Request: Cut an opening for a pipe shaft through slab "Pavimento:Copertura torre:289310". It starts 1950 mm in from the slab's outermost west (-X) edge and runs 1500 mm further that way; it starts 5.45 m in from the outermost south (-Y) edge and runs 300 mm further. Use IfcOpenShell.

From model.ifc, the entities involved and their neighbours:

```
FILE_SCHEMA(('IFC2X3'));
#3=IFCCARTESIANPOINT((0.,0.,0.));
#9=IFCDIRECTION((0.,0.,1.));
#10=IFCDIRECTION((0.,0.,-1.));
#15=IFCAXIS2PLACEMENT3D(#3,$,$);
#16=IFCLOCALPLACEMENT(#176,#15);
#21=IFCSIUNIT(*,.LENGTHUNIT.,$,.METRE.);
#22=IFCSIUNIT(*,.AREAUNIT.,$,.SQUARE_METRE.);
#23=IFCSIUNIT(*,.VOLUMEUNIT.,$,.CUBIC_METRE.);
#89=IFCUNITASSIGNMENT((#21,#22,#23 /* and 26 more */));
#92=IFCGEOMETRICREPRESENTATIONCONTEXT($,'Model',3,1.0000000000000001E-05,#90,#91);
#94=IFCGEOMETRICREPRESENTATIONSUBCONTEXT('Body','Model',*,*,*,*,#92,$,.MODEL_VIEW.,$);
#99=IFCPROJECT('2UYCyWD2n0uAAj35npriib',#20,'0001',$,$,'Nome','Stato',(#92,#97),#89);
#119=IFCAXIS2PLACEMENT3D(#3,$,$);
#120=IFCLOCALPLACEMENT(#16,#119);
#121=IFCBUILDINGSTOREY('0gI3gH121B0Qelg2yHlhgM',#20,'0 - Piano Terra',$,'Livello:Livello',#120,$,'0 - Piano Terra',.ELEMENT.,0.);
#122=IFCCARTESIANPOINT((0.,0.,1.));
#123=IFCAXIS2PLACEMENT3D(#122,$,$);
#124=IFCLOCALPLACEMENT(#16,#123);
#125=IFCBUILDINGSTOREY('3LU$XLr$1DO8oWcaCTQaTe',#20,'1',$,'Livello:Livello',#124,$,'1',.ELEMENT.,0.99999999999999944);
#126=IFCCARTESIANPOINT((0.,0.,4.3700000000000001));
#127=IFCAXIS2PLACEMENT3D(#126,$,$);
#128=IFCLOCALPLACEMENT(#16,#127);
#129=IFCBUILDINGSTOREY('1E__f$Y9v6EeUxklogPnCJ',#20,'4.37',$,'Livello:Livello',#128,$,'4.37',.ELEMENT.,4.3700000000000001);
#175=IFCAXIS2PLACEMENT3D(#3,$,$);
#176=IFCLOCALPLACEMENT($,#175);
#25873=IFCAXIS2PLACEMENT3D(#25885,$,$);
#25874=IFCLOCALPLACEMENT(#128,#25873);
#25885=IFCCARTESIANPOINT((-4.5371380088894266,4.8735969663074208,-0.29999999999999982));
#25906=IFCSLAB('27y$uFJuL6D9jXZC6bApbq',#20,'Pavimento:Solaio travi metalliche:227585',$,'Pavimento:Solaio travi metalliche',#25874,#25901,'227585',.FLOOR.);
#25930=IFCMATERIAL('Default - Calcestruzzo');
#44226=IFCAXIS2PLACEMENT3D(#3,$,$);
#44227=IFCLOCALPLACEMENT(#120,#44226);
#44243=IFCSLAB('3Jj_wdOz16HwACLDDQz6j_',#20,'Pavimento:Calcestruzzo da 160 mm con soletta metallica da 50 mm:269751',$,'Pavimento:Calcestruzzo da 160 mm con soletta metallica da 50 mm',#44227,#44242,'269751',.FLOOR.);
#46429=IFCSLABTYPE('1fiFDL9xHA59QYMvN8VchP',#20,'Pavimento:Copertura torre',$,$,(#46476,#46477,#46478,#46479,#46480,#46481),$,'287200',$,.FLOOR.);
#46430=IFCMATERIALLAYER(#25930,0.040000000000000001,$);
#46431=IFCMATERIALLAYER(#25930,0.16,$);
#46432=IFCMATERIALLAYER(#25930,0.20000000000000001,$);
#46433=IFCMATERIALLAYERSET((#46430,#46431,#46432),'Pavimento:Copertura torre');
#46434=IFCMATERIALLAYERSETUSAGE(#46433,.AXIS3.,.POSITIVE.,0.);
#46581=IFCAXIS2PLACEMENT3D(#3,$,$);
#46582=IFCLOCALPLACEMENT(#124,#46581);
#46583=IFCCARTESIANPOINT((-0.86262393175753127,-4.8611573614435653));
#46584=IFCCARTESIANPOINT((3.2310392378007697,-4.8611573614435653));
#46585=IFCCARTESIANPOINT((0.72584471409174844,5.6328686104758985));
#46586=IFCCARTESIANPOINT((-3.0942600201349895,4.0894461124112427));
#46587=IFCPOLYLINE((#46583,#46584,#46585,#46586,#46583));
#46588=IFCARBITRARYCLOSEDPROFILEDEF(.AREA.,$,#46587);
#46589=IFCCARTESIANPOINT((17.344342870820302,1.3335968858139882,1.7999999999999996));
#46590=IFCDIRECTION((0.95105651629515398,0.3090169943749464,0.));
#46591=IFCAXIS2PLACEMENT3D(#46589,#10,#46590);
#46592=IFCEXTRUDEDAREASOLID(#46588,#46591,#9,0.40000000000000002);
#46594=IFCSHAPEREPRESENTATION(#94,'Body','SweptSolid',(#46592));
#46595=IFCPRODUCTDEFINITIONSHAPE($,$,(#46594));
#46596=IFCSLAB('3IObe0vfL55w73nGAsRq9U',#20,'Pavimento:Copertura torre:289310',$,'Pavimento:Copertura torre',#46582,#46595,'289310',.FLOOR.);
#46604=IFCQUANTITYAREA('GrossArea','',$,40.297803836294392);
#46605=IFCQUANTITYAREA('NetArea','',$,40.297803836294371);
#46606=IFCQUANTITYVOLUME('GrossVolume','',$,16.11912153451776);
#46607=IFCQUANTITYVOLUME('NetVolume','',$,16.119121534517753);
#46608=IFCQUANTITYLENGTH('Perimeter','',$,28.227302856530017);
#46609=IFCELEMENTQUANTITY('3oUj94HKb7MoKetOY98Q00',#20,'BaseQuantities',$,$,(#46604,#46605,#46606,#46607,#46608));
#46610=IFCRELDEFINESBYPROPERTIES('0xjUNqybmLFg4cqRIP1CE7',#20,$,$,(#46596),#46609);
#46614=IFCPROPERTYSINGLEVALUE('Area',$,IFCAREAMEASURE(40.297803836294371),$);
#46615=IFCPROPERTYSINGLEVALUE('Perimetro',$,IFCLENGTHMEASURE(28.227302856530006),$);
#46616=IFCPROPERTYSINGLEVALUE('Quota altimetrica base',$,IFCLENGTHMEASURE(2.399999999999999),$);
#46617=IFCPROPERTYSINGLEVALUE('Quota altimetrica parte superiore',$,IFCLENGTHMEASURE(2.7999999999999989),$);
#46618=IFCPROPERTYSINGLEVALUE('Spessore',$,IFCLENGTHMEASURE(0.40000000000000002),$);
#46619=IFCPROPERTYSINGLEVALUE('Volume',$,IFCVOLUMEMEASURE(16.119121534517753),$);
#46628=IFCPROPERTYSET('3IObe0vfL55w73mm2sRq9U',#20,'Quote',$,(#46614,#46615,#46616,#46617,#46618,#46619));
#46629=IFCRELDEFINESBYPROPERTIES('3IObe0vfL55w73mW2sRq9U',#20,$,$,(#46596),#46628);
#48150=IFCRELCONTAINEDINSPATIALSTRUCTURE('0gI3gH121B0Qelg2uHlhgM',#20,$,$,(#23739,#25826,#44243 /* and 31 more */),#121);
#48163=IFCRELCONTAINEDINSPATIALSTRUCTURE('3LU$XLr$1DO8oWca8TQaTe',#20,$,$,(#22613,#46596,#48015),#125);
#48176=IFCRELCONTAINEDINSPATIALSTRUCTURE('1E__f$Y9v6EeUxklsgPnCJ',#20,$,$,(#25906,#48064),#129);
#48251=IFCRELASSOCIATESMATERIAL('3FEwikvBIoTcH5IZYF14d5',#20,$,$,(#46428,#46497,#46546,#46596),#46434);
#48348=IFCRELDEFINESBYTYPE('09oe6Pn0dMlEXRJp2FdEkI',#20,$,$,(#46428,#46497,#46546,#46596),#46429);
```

```python
import numpy as np
import ifcopenshell
import ifcopenshell.api.feature
import ifcopenshell.api.geometry
import ifcopenshell.api.pset
import ifcopenshell.api.root
import ifcopenshell.geom
import ifcopenshell.util.element
import ifcopenshell.util.placement
import ifcopenshell.util.representation
import ifcopenshell.util.shape
import ifcopenshell.util.unit

model = ifcopenshell.open("model.ifc")
unit_scale = ifcopenshell.util.unit.calculate_unit_scale(model)
area_scale = ifcopenshell.util.unit.calculate_unit_scale(model, "AREAUNIT")
volume_scale = ifcopenshell.util.unit.calculate_unit_scale(model, "VOLUMEUNIT")
settings = ifcopenshell.geom.settings()


def volume(element):
    """Net volume in cubic metres, openings subtracted."""
    shape = ifcopenshell.geom.create_shape(settings, element)
    return ifcopenshell.util.shape.get_volume(shape.geometry)


slab = model.by_guid("3IObe0vfL55w73nGAsRq9U")
before = volume(slab)

# Extent in the slab's own axes, in metres. The edges named are its -X and -Y sides.
slab_shape = ifcopenshell.geom.create_shape(settings, slab)
vertices = ifcopenshell.util.shape.get_vertices(slab_shape.geometry)
x_min, y_min, bottom = vertices.min(axis=0)
top = vertices[:, 2].max()

opening = ifcopenshell.api.root.create_entity(model, ifc_class="IfcOpeningElement", name="Pipe shaft opening")
context = ifcopenshell.util.representation.get_context(model, "Model", "Body", "MODEL_VIEW")
width, depth = 1.5, 0.3
outline = [(0.0, 0.0), (width, 0.0), (width, depth), (0.0, depth), (0.0, 0.0)]
# Overshoot both faces by 50 mm so the cut is clean.
shape = ifcopenshell.api.geometry.add_slab_representation(
    model, context=context, depth=top - bottom + 0.1, polyline=outline
)
ifcopenshell.api.geometry.assign_representation(model, product=opening, representation=shape)

matrix = ifcopenshell.util.placement.get_local_placement(slab.ObjectPlacement)
matrix[:, 3] = matrix @ np.append(np.array([x_min + 1.95, y_min + 5.45, bottom - 0.05]) / unit_scale, 1.0)
ifcopenshell.api.geometry.edit_object_placement(model, product=opening, matrix=matrix, is_si=False)
ifcopenshell.api.feature.add_feature(model, feature=opening, element=slab)

after = volume(slab)

# Update the slab's stored quantities.
qto = model.by_id(ifcopenshell.util.element.get_pset(slab, "BaseQuantities", should_inherit=False)["id"])
ifcopenshell.api.pset.edit_qto(model, qto=qto, properties={
    "NetArea": after / (top - bottom) / area_scale,
    "NetVolume": after / volume_scale,
})
pset = model.by_id(ifcopenshell.util.element.get_pset(slab, "Quote", should_inherit=False)["id"])
ifcopenshell.api.pset.edit_pset(model, pset=pset, properties={
    "Area": model.create_entity("IfcAreaMeasure", after / (top - bottom) / area_scale),
    "Volume": model.create_entity("IfcVolumeMeasure", after / volume_scale),
})

print(f"slab volume {before:.3f} -> {after:.3f} m3")

model.write("model_rev.ifc")
```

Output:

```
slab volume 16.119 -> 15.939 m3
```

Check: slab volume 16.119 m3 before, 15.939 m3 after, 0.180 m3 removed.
